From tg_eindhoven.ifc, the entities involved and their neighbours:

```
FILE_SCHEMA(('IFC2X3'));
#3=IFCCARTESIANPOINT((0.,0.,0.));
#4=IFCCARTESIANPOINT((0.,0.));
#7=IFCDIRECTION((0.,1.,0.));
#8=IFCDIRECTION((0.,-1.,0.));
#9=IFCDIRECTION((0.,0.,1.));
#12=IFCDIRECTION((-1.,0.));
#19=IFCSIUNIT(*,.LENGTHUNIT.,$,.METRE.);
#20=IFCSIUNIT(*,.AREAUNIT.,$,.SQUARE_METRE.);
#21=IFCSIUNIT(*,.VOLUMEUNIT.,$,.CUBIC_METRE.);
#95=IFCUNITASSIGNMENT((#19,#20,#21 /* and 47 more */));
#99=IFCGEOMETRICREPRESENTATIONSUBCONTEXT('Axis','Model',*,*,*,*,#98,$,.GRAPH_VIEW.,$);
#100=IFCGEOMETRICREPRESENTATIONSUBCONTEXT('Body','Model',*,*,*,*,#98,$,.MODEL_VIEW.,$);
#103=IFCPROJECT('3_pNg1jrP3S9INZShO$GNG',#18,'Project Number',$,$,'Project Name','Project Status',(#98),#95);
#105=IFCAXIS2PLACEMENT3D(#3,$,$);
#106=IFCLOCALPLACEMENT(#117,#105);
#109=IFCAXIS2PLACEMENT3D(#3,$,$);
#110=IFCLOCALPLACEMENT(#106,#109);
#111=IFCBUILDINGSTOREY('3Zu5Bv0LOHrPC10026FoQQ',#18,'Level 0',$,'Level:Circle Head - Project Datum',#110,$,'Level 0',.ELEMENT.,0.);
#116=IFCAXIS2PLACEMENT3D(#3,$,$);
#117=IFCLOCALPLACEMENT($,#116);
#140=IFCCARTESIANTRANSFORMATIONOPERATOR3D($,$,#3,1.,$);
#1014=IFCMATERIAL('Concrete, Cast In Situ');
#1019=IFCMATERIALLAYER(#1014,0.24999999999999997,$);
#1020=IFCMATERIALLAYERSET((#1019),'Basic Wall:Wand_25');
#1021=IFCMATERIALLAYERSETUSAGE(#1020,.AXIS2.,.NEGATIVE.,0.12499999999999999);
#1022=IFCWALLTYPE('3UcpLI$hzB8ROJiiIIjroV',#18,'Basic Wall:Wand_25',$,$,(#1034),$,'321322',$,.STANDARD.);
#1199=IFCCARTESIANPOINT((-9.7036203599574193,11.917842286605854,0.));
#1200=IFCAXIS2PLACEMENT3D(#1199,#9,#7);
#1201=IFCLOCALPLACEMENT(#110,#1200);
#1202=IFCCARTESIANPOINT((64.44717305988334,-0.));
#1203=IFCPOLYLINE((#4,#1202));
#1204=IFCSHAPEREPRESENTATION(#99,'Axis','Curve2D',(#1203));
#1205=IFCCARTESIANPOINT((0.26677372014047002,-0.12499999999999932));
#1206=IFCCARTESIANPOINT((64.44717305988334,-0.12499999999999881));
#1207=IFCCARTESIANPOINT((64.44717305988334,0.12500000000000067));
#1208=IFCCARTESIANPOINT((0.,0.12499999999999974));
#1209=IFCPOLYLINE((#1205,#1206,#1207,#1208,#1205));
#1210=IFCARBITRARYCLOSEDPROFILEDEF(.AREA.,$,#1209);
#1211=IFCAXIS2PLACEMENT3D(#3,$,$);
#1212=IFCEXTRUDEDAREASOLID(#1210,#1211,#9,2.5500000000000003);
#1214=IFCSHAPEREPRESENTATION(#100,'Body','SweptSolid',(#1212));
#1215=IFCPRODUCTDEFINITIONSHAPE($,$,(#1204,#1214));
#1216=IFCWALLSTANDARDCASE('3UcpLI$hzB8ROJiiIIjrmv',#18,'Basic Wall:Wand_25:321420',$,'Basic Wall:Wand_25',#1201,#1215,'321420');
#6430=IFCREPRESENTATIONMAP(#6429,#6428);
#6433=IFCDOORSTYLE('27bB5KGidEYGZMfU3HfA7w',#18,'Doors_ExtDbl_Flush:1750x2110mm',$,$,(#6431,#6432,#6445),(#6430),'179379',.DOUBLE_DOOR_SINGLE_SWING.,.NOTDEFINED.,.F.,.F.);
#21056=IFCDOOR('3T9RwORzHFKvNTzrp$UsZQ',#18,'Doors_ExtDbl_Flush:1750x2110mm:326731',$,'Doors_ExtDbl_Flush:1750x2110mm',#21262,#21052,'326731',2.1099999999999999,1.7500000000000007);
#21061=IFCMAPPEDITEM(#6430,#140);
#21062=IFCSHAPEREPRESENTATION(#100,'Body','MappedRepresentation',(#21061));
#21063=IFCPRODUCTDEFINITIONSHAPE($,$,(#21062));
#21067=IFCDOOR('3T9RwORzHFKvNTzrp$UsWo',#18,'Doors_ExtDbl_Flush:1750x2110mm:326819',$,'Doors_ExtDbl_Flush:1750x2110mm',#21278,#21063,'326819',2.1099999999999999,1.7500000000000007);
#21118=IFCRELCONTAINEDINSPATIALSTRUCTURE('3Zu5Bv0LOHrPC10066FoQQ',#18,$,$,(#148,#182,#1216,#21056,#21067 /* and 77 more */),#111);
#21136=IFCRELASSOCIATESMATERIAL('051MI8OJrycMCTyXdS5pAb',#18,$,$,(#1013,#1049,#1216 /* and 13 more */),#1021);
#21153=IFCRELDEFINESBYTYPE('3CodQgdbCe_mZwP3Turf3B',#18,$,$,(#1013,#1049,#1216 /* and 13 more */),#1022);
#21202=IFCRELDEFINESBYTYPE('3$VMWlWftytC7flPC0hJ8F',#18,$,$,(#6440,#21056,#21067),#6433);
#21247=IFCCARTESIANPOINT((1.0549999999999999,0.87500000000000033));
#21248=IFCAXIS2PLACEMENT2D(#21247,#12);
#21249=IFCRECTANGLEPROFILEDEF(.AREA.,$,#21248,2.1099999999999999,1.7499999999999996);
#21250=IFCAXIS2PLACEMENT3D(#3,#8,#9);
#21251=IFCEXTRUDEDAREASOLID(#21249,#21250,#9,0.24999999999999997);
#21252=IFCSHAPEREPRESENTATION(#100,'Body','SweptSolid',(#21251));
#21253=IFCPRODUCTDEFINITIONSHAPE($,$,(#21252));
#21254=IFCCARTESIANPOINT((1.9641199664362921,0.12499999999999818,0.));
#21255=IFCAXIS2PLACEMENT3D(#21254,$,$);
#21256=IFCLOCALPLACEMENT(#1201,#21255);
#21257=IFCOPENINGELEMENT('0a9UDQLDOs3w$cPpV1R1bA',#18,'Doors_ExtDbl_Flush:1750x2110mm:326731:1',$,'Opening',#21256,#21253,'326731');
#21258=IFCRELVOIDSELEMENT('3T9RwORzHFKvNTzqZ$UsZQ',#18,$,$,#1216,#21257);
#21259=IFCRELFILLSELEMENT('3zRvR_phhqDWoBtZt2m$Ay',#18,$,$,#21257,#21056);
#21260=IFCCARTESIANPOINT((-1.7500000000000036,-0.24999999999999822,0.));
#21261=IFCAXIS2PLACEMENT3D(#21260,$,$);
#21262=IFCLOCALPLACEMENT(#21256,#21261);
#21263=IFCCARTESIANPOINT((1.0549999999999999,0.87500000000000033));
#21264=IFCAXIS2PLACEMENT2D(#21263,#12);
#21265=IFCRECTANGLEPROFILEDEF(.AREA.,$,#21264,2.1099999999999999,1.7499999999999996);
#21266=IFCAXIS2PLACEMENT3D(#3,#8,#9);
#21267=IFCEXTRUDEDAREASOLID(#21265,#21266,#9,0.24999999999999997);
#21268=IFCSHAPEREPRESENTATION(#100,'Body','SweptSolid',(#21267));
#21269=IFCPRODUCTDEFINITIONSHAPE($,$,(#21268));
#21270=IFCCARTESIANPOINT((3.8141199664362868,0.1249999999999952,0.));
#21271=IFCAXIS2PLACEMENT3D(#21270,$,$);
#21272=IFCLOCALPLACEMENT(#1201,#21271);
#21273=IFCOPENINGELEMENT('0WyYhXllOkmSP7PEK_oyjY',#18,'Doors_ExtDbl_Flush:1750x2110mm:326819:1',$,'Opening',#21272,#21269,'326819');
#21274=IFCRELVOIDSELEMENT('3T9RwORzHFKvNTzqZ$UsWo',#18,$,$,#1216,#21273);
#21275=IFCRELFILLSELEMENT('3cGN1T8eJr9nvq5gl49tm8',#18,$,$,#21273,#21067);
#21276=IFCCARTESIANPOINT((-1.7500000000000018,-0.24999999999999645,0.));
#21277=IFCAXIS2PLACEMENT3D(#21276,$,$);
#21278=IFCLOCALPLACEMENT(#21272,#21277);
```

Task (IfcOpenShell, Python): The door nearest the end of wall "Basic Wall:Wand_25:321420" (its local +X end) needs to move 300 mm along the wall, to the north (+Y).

```python
import ifcopenshell
import ifcopenshell.api.geometry
import ifcopenshell.util.placement
import ifcopenshell.util.unit

model = ifcopenshell.open("tg_eindhoven.ifc")
unit_scale = ifcopenshell.util.unit.calculate_unit_scale(model)

door = model.by_guid("3T9RwORzHFKvNTzrp$UsWo")
opening = door.FillsVoids[0].RelatingOpeningElement
wall = opening.VoidsElements[0].RelatingBuildingElement

wall_matrix = ifcopenshell.util.placement.get_local_placement(wall.ObjectPlacement)
shift = wall_matrix[:3, 0] * 0.3 / unit_scale
before = ifcopenshell.util.placement.get_local_placement(door.ObjectPlacement)[:3, 3].copy()

# The door is placed relative to its opening, so it follows when the opening moves.
matrix = ifcopenshell.util.placement.get_local_placement(opening.ObjectPlacement)
matrix[:3, 3] += shift
ifcopenshell.api.geometry.edit_object_placement(
    model, product=opening, matrix=matrix, is_si=False, should_transform_children=True
)

after = ifcopenshell.util.placement.get_local_placement(door.ObjectPlacement)[:3, 3]
print("door moved by", (after - before).round(3) + 0.0)

model.write("tg_eindhoven_rev.ifc")
```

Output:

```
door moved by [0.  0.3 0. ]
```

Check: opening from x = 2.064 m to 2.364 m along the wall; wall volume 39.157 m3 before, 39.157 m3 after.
